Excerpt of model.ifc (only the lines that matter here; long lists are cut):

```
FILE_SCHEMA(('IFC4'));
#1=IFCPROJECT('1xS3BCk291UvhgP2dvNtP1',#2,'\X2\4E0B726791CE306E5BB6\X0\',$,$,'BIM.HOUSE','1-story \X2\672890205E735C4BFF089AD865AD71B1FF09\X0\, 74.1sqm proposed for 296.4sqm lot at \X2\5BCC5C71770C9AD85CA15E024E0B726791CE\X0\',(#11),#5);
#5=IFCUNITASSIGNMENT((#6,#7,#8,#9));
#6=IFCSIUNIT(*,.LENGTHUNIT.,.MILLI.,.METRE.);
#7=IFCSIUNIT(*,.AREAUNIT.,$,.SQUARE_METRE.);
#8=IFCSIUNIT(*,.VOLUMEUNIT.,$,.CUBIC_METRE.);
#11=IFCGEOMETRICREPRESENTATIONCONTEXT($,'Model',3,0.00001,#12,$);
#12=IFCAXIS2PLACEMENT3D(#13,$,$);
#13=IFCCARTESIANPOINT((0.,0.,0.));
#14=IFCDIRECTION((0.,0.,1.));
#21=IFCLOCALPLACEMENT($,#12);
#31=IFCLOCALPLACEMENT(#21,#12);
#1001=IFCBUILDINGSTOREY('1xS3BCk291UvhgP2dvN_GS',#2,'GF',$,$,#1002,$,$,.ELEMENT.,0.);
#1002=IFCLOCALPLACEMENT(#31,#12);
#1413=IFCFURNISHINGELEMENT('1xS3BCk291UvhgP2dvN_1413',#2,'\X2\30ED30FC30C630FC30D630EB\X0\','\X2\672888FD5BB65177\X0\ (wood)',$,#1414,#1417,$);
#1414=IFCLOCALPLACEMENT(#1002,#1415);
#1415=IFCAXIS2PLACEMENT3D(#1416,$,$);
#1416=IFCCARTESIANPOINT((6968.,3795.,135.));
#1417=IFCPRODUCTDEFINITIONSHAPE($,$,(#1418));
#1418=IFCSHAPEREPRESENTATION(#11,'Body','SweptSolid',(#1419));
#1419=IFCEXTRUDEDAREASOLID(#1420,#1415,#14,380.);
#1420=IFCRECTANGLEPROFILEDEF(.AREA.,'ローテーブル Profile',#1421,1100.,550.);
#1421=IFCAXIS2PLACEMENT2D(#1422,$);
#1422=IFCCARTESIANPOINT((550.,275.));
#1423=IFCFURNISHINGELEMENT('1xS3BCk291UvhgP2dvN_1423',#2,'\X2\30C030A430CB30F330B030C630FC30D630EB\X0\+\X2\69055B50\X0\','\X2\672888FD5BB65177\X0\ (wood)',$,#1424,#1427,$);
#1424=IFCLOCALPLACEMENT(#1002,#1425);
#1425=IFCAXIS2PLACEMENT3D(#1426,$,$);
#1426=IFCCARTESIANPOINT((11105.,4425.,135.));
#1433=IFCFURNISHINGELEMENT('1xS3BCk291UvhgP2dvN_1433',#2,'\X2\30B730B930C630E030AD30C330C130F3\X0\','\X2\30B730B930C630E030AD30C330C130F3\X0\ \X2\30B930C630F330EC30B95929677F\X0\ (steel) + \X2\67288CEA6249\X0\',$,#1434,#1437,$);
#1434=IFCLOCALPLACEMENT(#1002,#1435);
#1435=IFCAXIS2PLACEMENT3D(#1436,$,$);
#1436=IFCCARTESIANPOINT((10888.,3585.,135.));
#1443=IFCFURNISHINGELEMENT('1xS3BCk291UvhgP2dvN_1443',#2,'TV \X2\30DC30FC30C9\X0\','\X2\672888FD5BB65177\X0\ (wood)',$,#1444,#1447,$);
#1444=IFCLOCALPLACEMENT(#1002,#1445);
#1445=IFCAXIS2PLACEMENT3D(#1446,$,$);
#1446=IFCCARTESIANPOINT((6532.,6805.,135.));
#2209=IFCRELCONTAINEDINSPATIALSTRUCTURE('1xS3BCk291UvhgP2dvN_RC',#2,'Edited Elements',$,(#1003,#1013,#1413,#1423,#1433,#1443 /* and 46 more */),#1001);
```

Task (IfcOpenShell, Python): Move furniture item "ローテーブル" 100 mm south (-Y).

```python
import ifcopenshell
import ifcopenshell.api.geometry
import ifcopenshell.util.placement
import ifcopenshell.util.unit

model = ifcopenshell.open("model.ifc")
unit_scale = ifcopenshell.util.unit.calculate_unit_scale(model)

item = model.by_id(1413)
matrix = ifcopenshell.util.placement.get_local_placement(item.ObjectPlacement)
matrix[1, 3] -= 0.1 / unit_scale
ifcopenshell.api.geometry.edit_object_placement(model, product=item, matrix=matrix, is_si=False)

print(ifcopenshell.util.placement.get_local_placement(item.ObjectPlacement).round(3) + 0.0)

model.write("model_updated.ifc")
```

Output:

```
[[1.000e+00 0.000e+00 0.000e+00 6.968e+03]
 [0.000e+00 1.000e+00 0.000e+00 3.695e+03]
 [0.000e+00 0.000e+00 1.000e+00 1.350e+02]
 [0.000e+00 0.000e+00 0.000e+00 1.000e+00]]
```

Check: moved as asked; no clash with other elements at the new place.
